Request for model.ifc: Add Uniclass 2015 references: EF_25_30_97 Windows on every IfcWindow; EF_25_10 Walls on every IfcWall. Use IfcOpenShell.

First a look at what the model holds.

```python
import ifcopenshell

model = ifcopenshell.open("model.ifc")
print(model.schema)
print("classifications:", [c.Name for c in model.by_type("IfcClassification")])
for ifc_class in ("IfcDoor", "IfcRoof", "IfcStair", "IfcWall", "IfcWindow"):
    print(ifc_class, len(model.by_type(ifc_class)))
```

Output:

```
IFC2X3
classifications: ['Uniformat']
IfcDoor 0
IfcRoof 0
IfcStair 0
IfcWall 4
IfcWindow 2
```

```python
import ifcopenshell
import ifcopenshell.api.classification

model = ifcopenshell.open("model.ifc")

# IFC2X3 requires Source and Edition and has no link from the project to the system.
system = model.create_entity("IfcClassification", Source="NBS", Edition="2015", Name="Uniclass 2015")

codes = {
    "IfcWindow": ("EF_25_30_97", "Windows"),
    "IfcWall": ("EF_25_10", "Walls"),
}
for ifc_class, (code, name) in codes.items():
    products = model.by_type(ifc_class)
    ifcopenshell.api.classification.add_reference(
        model, products=products, classification=system, identification=code, name=name
    )
    print(code, len(products))

model.write("model_edited.ifc")
```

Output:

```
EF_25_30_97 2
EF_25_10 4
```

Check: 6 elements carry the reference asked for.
